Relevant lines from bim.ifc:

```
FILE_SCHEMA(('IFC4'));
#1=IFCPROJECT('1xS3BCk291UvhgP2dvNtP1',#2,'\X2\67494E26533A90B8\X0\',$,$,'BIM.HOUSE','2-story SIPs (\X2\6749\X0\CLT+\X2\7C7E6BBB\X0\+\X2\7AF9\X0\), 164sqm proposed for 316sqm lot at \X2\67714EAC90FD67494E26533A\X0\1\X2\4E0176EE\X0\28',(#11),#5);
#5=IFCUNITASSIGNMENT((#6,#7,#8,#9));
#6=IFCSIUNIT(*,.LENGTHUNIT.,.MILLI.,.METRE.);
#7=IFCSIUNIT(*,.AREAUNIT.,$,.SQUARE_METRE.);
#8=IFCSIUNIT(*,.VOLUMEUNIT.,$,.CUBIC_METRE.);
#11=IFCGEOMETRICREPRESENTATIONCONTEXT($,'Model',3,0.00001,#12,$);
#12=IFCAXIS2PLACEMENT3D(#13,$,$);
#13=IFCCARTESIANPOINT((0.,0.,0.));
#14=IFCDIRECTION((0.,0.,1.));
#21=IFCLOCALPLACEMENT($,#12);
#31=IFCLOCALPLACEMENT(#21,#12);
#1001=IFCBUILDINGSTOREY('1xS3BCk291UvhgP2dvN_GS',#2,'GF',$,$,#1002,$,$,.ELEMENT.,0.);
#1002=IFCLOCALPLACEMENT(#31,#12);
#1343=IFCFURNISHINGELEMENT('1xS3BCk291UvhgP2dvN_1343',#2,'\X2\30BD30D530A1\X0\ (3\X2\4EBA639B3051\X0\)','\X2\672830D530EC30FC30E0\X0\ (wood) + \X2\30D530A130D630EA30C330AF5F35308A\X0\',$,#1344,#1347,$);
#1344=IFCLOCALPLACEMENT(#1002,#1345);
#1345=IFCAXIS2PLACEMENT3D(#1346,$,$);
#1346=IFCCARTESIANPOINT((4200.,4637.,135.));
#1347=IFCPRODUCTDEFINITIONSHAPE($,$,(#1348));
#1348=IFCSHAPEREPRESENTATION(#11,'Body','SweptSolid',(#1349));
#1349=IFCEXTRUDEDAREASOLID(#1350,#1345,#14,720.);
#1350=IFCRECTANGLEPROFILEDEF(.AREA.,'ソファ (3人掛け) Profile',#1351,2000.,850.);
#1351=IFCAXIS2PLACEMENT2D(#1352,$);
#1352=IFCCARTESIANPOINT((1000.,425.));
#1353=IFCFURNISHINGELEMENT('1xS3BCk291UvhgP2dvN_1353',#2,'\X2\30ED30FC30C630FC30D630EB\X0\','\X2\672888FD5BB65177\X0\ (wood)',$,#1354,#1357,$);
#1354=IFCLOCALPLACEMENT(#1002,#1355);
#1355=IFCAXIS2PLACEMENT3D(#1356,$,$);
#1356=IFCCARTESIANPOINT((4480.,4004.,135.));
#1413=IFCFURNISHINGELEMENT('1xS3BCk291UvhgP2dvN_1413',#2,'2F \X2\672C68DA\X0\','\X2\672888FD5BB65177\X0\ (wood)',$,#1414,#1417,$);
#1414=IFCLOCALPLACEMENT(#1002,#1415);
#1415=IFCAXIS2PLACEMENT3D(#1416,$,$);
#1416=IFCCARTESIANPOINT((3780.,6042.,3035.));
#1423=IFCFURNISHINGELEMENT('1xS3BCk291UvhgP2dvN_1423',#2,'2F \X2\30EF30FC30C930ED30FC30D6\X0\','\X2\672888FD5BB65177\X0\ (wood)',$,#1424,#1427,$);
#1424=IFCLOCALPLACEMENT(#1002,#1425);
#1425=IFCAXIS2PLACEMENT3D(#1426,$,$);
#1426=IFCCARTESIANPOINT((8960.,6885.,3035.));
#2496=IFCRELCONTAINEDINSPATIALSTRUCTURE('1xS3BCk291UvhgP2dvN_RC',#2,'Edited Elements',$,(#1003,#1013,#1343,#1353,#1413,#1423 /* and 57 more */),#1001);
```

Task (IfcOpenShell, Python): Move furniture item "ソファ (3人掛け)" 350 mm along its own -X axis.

```python
import ifcopenshell
import ifcopenshell.api.geometry
import ifcopenshell.util.placement
import ifcopenshell.util.unit

model = ifcopenshell.open("bim.ifc")
unit_scale = ifcopenshell.util.unit.calculate_unit_scale(model)

item = model.by_guid("1xS3BCk291UvhgP2dvN_1343")
matrix = ifcopenshell.util.placement.get_local_placement(item.ObjectPlacement)
matrix[:3, 3] -= matrix[:3, 0] * 0.35 / unit_scale
ifcopenshell.api.geometry.edit_object_placement(model, product=item, matrix=matrix, is_si=False)

print(ifcopenshell.util.placement.get_local_placement(item.ObjectPlacement).round(3) + 0.0)

model.write("bim-out.ifc")
```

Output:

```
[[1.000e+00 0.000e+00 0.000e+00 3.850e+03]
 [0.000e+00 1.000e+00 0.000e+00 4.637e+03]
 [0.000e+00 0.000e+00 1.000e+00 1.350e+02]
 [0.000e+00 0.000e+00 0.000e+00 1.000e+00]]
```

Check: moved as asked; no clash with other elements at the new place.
